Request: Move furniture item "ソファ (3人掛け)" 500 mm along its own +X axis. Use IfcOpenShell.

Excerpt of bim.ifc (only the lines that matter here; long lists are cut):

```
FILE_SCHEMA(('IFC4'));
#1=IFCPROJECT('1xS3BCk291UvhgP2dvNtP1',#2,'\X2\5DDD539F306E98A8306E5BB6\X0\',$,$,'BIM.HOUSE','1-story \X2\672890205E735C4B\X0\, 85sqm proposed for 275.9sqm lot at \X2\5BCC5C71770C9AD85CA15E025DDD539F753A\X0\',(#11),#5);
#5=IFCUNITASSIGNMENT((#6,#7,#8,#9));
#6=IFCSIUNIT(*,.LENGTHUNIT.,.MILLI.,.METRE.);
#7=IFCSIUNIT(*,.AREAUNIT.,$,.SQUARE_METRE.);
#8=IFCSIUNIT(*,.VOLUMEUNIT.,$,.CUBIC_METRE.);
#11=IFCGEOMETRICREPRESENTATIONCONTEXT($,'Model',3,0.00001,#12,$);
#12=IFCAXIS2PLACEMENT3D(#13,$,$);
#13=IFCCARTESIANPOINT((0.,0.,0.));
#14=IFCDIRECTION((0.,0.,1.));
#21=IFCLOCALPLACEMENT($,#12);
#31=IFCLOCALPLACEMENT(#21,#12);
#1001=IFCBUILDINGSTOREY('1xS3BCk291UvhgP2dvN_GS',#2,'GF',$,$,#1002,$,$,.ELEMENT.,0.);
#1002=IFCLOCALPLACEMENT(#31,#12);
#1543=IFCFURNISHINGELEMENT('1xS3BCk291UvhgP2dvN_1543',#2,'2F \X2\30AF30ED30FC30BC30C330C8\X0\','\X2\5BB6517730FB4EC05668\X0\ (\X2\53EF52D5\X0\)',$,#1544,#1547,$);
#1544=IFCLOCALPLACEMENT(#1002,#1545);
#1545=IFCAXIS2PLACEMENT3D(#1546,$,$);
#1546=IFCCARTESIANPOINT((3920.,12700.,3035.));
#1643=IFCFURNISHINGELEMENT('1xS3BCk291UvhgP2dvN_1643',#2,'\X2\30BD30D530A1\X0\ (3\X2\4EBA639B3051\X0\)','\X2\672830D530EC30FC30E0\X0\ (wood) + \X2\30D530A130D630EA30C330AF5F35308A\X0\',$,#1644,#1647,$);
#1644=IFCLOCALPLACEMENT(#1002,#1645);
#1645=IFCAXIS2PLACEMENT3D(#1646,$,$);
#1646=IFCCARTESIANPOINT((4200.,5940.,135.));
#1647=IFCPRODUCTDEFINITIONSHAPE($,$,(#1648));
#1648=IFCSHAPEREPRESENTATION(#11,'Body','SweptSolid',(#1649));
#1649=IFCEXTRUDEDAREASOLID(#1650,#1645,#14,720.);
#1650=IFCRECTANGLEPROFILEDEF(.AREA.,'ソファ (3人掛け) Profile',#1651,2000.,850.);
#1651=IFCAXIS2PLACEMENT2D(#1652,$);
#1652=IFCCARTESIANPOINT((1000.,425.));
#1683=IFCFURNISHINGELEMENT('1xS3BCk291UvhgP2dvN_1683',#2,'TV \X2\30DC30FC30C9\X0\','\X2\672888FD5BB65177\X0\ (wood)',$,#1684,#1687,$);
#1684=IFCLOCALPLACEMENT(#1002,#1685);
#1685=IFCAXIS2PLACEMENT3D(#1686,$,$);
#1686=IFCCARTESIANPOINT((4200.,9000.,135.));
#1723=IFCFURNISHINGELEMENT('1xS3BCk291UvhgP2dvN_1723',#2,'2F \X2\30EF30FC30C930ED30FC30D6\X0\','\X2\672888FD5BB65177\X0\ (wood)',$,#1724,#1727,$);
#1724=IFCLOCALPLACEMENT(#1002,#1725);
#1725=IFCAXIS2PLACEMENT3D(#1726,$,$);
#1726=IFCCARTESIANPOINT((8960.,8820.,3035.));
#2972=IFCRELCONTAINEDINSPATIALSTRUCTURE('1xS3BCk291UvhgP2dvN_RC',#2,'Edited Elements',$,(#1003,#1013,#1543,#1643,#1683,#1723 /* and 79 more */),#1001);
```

```python
import ifcopenshell
import ifcopenshell.api.geometry
import ifcopenshell.util.placement

model = ifcopenshell.open("bim.ifc")

item = model.by_guid("1xS3BCk291UvhgP2dvN_1643")
matrix = ifcopenshell.util.placement.get_local_placement(item.ObjectPlacement)
matrix[:3, 3] += matrix[:3, 0] * 500.0
ifcopenshell.api.geometry.edit_object_placement(model, product=item, matrix=matrix, is_si=False)

print(ifcopenshell.util.placement.get_local_placement(item.ObjectPlacement).round(3) + 0.0)

model.write("bim_updated.ifc")
```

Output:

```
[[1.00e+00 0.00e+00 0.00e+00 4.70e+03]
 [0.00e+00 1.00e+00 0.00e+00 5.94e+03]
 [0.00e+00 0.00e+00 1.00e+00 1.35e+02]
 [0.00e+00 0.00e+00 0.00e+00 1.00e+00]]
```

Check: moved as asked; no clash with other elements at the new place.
